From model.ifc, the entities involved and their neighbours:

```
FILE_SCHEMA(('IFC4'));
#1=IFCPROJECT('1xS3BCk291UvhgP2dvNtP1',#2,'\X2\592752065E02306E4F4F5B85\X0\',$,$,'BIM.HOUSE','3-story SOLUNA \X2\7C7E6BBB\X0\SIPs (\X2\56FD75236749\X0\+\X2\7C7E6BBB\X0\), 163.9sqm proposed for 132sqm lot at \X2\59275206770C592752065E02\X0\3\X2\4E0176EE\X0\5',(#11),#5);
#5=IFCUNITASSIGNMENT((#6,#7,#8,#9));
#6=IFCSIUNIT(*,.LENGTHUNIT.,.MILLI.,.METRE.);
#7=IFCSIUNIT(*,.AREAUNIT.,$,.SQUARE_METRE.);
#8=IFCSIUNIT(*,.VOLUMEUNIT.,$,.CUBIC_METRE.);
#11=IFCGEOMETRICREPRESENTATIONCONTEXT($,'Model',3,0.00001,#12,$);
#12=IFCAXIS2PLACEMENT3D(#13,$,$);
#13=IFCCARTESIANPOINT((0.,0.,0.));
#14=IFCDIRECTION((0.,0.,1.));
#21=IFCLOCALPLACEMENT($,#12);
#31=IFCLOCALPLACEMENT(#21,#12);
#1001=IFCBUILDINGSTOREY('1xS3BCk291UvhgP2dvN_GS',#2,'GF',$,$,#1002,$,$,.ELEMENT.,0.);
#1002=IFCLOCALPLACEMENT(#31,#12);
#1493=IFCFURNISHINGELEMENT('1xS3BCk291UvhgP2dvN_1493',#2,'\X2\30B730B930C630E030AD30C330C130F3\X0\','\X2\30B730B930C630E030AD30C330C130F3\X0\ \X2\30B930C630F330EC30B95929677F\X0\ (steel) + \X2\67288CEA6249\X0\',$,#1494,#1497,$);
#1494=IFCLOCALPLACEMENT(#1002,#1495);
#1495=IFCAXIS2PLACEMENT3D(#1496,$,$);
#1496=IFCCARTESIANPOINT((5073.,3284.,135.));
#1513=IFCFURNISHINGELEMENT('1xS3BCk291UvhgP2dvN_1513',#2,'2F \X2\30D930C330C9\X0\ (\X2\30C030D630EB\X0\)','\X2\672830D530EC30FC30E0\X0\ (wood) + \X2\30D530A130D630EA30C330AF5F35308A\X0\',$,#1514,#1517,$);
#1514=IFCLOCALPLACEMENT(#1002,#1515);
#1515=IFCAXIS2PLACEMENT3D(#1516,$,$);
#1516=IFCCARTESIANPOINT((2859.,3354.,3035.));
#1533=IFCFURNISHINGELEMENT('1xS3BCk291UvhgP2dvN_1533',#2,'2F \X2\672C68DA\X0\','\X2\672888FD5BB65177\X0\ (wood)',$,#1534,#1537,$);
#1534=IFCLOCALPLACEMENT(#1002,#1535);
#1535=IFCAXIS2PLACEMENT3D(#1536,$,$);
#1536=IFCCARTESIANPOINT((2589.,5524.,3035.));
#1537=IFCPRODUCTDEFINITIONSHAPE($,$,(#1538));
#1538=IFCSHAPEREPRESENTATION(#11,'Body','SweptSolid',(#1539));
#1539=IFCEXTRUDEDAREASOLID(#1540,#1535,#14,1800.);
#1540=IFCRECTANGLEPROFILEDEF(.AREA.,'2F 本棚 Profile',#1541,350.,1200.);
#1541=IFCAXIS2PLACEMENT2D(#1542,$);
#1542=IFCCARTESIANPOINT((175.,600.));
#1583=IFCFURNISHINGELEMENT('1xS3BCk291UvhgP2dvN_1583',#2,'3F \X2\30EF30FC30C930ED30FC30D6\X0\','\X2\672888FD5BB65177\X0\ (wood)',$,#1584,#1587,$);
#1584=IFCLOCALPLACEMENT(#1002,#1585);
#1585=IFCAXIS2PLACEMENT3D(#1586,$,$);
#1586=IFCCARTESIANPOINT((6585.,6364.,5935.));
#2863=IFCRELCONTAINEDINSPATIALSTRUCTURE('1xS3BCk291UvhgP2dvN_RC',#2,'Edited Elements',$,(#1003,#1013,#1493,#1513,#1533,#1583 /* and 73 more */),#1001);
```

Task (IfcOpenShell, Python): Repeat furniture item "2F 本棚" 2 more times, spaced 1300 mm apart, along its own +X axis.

```python
import ifcopenshell
import ifcopenshell.api.geometry
import ifcopenshell.api.root
import ifcopenshell.util.element
import ifcopenshell.util.placement

model = ifcopenshell.open("model.ifc")


def reuse_history(source, copy):
    """copy_class also copies each property set's owner history, people and application; keep the originals."""
    for rel in copy.IsDefinedBy:
        if rel.is_a("IfcRelDefinesByProperties") and (history := rel.RelatingPropertyDefinition.OwnerHistory):
            rel.RelatingPropertyDefinition.OwnerHistory = source.OwnerHistory
            ifcopenshell.util.element.remove_deep2(model, history)


source = model.by_guid("1xS3BCk291UvhgP2dvN_1533")
base = ifcopenshell.util.placement.get_local_placement(source.ObjectPlacement)
step = base[:3, 0] * 1300.0

for i in range(1, 3):
    copy = ifcopenshell.api.root.copy_class(model, product=source)
    copy.Representation = ifcopenshell.util.element.copy_deep(
        model, source.Representation, exclude=["IfcGeometricRepresentationContext", "IfcRepresentationMap"]
    )
    reuse_history(source, copy)
    matrix = base.copy()
    matrix[:3, 3] += i * step
    print("added at", matrix[:3, 3].round(3) + 0.0)
    ifcopenshell.api.geometry.edit_object_placement(model, product=copy, matrix=matrix, is_si=False)

model.write("model_v2.ifc")
```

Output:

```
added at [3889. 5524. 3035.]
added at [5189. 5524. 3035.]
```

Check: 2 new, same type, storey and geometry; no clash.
